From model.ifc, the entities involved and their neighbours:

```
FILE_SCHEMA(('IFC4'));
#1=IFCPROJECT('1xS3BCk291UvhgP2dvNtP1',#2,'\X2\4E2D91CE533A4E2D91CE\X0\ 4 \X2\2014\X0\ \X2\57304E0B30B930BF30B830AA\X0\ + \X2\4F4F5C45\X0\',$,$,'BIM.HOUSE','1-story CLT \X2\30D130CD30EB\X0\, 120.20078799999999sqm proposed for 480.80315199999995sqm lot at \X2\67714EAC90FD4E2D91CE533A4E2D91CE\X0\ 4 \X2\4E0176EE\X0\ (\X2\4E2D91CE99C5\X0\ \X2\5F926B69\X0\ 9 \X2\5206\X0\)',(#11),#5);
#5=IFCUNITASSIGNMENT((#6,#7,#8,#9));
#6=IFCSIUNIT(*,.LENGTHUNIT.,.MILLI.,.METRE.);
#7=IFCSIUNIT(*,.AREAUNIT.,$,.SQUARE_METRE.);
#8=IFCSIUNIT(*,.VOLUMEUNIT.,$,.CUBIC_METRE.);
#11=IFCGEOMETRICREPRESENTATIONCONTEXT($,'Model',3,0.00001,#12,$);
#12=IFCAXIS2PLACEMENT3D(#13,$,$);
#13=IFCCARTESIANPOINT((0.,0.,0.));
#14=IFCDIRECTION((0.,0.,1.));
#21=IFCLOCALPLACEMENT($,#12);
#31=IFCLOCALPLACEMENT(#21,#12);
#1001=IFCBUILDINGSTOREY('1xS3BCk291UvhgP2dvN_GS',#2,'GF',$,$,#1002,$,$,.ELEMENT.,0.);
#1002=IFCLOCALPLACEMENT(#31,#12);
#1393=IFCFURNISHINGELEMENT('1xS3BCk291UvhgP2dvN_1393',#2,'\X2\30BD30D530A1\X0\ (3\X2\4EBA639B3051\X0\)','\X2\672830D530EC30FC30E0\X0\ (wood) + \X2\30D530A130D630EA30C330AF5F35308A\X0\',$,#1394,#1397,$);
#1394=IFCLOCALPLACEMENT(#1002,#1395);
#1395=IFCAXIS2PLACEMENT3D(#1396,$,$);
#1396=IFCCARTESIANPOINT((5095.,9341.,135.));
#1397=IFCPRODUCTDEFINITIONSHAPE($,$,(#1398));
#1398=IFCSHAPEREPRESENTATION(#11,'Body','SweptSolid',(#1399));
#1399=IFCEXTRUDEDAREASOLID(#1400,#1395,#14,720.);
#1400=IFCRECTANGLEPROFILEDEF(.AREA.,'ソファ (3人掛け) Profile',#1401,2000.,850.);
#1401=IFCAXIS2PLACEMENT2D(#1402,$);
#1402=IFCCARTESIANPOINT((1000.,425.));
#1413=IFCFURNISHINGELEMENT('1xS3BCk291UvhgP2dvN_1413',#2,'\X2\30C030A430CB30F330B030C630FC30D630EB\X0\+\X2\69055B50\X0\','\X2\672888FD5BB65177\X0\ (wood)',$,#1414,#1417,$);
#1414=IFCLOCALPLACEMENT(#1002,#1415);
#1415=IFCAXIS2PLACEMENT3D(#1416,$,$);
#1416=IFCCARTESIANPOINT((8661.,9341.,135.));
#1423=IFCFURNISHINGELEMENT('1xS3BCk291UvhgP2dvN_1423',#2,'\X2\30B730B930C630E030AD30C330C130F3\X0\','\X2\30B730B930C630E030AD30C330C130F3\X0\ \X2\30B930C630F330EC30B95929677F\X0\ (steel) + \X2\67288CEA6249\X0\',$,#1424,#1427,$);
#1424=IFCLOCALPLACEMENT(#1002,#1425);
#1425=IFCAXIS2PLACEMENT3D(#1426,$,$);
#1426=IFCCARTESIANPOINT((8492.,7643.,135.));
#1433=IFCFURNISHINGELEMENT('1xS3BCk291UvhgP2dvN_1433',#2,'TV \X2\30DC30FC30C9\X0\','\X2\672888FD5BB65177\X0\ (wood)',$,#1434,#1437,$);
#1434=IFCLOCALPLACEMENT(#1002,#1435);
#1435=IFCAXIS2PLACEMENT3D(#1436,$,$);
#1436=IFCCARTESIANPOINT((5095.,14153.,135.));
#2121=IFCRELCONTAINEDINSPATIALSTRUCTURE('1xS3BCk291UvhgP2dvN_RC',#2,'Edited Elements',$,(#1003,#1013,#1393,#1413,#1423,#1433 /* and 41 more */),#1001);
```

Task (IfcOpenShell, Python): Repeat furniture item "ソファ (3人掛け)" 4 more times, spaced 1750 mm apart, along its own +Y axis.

```python
import ifcopenshell
import ifcopenshell.api.geometry
import ifcopenshell.api.root
import ifcopenshell.util.element
import ifcopenshell.util.placement
import ifcopenshell.util.unit

model = ifcopenshell.open("model.ifc")
unit_scale = ifcopenshell.util.unit.calculate_unit_scale(model)


def reuse_history(source, copy):
    """copy_class also copies each property set's owner history, people and application; keep the originals."""
    for rel in copy.IsDefinedBy:
        if rel.is_a("IfcRelDefinesByProperties") and (history := rel.RelatingPropertyDefinition.OwnerHistory):
            rel.RelatingPropertyDefinition.OwnerHistory = source.OwnerHistory
            ifcopenshell.util.element.remove_deep2(model, history)


source = model.by_id(1393)
base = ifcopenshell.util.placement.get_local_placement(source.ObjectPlacement)
step = base[:3, 1] * 1.75 / unit_scale

for i in range(1, 5):
    copy = ifcopenshell.api.root.copy_class(model, product=source)
    copy.Representation = ifcopenshell.util.element.copy_deep(
        model, source.Representation, exclude=["IfcGeometricRepresentationContext", "IfcRepresentationMap"]
    )
    reuse_history(source, copy)
    matrix = base.copy()
    matrix[:3, 3] += i * step
    print("added at", matrix[:3, 3].round(3) + 0.0)
    ifcopenshell.api.geometry.edit_object_placement(model, product=copy, matrix=matrix, is_si=False)

model.write("model_edited.ifc")
```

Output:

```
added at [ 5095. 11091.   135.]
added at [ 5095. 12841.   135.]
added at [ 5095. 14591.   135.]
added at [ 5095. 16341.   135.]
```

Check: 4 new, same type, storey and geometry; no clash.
